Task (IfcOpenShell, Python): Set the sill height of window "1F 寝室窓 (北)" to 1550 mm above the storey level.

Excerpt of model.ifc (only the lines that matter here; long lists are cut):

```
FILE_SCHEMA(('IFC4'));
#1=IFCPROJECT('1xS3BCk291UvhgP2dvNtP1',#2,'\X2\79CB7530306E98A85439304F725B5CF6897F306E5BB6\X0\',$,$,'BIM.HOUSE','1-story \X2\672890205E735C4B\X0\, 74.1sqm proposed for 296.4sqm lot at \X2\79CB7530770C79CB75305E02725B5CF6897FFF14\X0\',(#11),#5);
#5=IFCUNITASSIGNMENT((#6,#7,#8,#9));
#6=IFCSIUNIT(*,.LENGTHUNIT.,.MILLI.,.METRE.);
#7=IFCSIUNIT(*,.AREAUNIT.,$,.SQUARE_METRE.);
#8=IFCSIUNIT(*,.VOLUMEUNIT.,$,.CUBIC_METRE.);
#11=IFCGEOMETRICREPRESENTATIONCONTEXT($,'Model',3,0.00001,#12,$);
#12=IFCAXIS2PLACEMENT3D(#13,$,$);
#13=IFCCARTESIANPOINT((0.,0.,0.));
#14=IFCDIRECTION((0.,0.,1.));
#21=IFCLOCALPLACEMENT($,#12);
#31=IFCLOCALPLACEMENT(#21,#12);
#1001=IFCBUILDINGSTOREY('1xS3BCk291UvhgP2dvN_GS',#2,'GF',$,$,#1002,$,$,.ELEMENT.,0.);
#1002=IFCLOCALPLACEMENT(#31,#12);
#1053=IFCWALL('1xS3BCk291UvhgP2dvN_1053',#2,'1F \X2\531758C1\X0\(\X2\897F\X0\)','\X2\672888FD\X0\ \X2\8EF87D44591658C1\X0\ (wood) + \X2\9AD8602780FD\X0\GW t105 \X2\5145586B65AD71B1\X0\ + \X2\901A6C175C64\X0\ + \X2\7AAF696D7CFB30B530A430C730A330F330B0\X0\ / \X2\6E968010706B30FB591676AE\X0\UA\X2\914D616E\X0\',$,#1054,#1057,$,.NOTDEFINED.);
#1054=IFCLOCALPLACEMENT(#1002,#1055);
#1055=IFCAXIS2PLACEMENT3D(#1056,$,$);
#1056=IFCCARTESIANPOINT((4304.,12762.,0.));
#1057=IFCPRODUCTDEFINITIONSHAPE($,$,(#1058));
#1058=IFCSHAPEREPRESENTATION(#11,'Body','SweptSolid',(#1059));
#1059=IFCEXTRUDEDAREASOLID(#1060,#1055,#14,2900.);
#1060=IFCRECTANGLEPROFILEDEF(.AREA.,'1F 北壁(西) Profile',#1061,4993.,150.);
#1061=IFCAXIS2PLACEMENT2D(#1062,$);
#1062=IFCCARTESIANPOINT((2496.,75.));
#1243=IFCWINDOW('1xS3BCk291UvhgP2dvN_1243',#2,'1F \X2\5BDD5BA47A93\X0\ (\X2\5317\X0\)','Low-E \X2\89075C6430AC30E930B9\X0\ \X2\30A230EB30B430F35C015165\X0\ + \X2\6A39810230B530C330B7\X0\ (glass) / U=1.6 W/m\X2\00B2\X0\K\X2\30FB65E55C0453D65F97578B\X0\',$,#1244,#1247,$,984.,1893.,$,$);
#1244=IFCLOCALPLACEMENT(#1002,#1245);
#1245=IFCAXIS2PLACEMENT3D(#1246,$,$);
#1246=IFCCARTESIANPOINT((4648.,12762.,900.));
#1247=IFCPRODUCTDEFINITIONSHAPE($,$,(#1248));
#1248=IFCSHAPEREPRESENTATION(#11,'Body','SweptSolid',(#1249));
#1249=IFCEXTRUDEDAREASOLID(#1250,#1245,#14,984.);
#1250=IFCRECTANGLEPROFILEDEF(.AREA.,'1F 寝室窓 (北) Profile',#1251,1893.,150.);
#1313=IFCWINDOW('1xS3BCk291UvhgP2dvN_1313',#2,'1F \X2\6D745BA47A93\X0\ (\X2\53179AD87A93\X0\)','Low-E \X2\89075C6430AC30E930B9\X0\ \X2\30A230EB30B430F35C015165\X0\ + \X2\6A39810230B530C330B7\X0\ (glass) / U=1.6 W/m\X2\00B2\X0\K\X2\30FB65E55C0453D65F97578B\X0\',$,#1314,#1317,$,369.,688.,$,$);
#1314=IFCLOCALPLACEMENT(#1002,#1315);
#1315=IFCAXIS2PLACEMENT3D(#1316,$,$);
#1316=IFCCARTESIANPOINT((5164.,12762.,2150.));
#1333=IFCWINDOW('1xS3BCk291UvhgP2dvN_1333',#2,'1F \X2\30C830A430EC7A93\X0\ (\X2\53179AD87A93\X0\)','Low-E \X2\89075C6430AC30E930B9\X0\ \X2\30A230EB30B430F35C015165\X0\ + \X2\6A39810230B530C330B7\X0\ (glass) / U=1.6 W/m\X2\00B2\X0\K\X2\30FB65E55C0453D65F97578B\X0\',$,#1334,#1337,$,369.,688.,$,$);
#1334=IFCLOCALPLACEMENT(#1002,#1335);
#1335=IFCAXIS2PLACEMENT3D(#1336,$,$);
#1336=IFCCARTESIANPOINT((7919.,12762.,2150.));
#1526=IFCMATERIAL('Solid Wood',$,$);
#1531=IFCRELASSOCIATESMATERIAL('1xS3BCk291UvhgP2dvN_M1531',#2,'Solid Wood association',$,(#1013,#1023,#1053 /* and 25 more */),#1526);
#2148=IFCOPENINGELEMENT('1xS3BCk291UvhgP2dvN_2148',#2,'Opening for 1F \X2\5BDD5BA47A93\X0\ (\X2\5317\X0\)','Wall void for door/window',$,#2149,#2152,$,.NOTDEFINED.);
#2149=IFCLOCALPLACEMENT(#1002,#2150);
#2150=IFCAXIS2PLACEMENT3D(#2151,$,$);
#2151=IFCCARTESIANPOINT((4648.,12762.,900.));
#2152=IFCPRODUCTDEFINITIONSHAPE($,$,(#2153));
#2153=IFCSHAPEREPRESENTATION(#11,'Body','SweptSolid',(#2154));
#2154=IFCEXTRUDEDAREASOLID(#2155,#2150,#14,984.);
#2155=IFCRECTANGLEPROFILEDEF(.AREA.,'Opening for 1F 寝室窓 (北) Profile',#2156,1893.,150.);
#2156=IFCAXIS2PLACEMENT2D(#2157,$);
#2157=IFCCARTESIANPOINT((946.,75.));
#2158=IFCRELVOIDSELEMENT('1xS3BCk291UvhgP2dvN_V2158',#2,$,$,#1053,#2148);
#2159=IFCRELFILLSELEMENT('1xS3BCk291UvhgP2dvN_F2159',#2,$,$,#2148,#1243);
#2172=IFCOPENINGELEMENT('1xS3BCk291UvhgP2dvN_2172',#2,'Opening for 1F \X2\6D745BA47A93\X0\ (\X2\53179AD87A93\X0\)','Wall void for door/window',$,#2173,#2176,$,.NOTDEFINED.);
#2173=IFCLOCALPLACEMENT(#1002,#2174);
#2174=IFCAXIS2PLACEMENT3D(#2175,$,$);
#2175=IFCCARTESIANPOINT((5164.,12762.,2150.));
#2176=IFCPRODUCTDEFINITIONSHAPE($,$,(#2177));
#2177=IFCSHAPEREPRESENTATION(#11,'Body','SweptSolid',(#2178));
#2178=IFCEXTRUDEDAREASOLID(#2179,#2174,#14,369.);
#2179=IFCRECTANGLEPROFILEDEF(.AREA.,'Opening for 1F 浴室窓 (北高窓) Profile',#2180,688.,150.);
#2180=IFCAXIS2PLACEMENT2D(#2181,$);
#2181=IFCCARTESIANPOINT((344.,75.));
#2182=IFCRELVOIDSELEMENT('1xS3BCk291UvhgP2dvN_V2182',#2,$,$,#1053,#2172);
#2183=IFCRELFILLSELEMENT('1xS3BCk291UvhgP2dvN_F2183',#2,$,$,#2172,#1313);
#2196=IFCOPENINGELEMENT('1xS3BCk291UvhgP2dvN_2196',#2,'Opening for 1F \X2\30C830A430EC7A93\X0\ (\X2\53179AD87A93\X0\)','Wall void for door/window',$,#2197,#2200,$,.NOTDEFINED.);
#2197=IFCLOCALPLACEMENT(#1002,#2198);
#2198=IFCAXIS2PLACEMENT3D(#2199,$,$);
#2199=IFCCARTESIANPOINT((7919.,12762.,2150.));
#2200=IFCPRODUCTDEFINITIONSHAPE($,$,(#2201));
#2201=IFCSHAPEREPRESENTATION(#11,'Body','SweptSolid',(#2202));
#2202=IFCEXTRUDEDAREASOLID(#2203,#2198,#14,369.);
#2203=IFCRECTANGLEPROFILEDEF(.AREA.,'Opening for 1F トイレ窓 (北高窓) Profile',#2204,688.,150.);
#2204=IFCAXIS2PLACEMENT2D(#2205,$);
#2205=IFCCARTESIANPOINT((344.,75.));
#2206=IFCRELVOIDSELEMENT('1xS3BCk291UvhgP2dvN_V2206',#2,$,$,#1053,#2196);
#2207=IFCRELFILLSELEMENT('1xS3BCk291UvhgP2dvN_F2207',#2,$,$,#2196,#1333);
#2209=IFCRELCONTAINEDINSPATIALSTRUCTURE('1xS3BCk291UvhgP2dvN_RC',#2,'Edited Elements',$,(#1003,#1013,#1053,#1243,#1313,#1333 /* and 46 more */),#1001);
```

```python
import numpy as np
import ifcopenshell
import ifcopenshell.api.geometry
import ifcopenshell.geom
import ifcopenshell.util.element
import ifcopenshell.util.placement
import ifcopenshell.util.shape
import ifcopenshell.util.unit

model = ifcopenshell.open("model.ifc")
unit_scale = ifcopenshell.util.unit.calculate_unit_scale(model)

window = model.by_guid("1xS3BCk291UvhgP2dvN_1243")
opening = window.FillsVoids[0].RelatingOpeningElement
storey = ifcopenshell.util.element.get_container(window, ifc_class="IfcBuildingStorey")
level = ifcopenshell.util.placement.get_local_placement(storey.ObjectPlacement)[2, 3]

# The opening's origin need not be at the sill, so measure its lowest point.
shape = ifcopenshell.geom.create_shape(ifcopenshell.geom.settings(), opening)
bottom = ifcopenshell.util.shape.get_shape_bottom_elevation(shape, shape.geometry) / unit_scale
dz = level + 1550.0 - bottom

shift = np.array([0.0, 0.0, dz])
# The window is not placed relative to its opening, so move both.
for product in (opening, window):
    matrix = ifcopenshell.util.placement.get_local_placement(product.ObjectPlacement)
    matrix[:3, 3] += shift
    ifcopenshell.api.geometry.edit_object_placement(model, product=product, matrix=matrix, is_si=False)

print(f"moved by {dz * unit_scale:+.3f} m")

model.write("model_updated.ifc")
```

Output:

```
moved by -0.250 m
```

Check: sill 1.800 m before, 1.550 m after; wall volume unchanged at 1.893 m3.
